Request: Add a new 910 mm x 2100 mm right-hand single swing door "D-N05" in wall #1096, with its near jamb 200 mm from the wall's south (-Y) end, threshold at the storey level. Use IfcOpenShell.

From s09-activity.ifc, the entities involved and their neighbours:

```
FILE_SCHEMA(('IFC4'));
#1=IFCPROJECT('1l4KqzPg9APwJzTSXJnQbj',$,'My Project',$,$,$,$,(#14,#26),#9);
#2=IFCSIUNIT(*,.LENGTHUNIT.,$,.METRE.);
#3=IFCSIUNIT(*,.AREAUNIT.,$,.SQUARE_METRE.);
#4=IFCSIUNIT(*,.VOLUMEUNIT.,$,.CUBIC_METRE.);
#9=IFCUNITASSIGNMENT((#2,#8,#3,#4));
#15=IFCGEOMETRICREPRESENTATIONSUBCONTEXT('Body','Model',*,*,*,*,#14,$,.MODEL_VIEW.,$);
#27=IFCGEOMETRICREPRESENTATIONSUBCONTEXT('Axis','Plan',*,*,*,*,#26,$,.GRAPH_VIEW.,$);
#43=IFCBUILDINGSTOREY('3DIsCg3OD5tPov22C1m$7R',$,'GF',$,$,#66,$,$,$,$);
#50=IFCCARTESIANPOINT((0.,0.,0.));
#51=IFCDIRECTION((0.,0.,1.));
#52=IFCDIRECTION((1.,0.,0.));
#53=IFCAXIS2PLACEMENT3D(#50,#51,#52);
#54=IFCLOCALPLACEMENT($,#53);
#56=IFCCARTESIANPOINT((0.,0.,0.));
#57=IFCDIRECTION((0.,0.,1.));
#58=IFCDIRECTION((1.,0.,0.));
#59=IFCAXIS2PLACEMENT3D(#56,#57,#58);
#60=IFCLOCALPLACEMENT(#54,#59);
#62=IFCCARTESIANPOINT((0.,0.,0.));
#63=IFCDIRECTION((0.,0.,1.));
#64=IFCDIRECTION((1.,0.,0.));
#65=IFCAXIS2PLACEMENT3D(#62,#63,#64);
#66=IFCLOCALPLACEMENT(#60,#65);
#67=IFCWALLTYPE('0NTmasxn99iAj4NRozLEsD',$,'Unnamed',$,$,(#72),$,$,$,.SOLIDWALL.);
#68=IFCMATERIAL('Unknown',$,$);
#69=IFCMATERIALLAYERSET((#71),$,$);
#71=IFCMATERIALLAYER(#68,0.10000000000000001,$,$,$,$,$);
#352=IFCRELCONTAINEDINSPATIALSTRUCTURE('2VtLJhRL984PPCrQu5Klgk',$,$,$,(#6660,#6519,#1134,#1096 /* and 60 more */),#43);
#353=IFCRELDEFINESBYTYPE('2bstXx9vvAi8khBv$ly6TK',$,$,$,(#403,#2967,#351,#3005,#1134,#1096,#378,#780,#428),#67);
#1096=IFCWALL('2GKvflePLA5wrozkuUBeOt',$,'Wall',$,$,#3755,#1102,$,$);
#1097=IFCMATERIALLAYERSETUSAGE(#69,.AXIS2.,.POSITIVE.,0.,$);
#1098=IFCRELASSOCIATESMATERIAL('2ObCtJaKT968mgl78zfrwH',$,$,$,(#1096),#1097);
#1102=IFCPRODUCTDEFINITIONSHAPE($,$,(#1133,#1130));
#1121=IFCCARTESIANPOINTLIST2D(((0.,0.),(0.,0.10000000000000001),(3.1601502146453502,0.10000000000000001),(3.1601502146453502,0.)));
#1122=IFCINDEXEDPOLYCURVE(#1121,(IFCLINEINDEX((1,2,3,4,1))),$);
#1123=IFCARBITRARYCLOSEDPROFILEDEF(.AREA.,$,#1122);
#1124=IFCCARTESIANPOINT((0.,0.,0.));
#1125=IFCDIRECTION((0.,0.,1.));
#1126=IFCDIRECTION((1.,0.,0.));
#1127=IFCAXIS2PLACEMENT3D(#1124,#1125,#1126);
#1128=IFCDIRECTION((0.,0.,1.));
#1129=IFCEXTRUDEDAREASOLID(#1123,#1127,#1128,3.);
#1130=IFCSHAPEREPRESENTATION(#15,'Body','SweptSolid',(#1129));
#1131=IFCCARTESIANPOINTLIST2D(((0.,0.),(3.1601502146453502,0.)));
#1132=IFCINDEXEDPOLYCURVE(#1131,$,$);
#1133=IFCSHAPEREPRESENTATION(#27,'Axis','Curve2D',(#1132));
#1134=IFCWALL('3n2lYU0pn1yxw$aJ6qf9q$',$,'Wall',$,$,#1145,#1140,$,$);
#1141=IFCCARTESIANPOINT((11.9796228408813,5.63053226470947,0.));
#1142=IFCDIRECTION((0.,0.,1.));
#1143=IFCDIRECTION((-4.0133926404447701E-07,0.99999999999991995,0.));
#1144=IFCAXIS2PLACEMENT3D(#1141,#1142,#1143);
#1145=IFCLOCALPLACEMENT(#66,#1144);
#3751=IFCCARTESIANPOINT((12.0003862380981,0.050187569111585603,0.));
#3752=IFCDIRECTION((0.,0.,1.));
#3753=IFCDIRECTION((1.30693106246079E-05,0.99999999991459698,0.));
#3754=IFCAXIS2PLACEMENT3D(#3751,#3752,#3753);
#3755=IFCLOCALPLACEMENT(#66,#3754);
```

```python
import numpy as np
import ifcopenshell
import ifcopenshell.api.feature
import ifcopenshell.api.geometry
import ifcopenshell.api.root
import ifcopenshell.api.spatial
import ifcopenshell.geom
import ifcopenshell.util.element
import ifcopenshell.util.placement
import ifcopenshell.util.representation
import ifcopenshell.util.shape
import ifcopenshell.util.unit

model = ifcopenshell.open("s09-activity.ifc")
unit_scale = ifcopenshell.util.unit.calculate_unit_scale(model)
settings = ifcopenshell.geom.settings()


def volume(element):
    """Net volume in cubic metres, openings subtracted."""
    shape = ifcopenshell.geom.create_shape(settings, element)
    return ifcopenshell.util.shape.get_volume(shape.geometry)


wall = model.by_guid("2GKvflePLA5wrozkuUBeOt")
storey = ifcopenshell.util.element.get_container(wall, ifc_class="IfcBuildingStorey")
context = ifcopenshell.util.representation.get_context(model, "Model", "Body", "MODEL_VIEW")
before = volume(wall)

width, height, from_end, sill = 0.91, 2.1, 0.2, 0.0  # metres

# The wall runs along its own X axis, and the end named is its -X end.
wall_shape = ifcopenshell.geom.create_shape(settings, wall)
x, y, z = ifcopenshell.util.shape.get_vertices(wall_shape.geometry).T
start = x.min() + from_end
face, thickness = float(y.min()), float(y.max() - y.min())
wall_matrix = ifcopenshell.util.placement.get_local_placement(wall.ObjectPlacement)
level = ifcopenshell.util.placement.get_local_placement(storey.ObjectPlacement)[2, 3]


def in_wall(x, y):
    """Placement at x, y metres in the wall's axes, at sill height."""
    matrix = wall_matrix.copy()
    matrix[:, 3] = wall_matrix @ np.array([x / unit_scale, y / unit_scale, 0.0, 1.0])
    matrix[2, 3] = level + sill / unit_scale
    return matrix


# Opening: a box that overshoots both wall faces by 50 mm.
opening = ifcopenshell.api.root.create_entity(model, ifc_class="IfcOpeningElement", predefined_type="OPENING")
box = ifcopenshell.api.geometry.add_wall_representation(
    model, context=context, length=width, height=height, thickness=thickness + 0.1
)
ifcopenshell.api.geometry.assign_representation(model, product=opening, representation=box)
ifcopenshell.api.geometry.edit_object_placement(model, product=opening, matrix=in_wall(start, face - 0.05), is_si=False)
ifcopenshell.api.feature.add_feature(model, feature=opening, element=wall)

door = ifcopenshell.api.root.create_entity(model, ifc_class="IfcDoor", name="D-N05", predefined_type="DOOR")
door.OverallWidth, door.OverallHeight = width / unit_scale, height / unit_scale
door.OperationType = "SINGLE_SWING_RIGHT"
body = ifcopenshell.api.geometry.add_door_representation(
    model,
    context=context,
    overall_width=door.OverallWidth,
    overall_height=door.OverallHeight,
    operation_type="SINGLE_SWING_RIGHT",
    lining_properties={"LiningDepth": thickness / unit_scale, "ThresholdDepth": thickness / unit_scale},
)
ifcopenshell.api.geometry.assign_representation(model, product=door, representation=body)
ifcopenshell.api.spatial.assign_container(model, products=[door], relating_structure=storey)
ifcopenshell.api.feature.add_filling(model, opening=opening, element=door)

# The lining spans the wall, so the door starts at the wall face.
ifcopenshell.api.geometry.edit_object_placement(model, product=door, matrix=in_wall(start, face), is_si=False)

after = volume(wall)

print(f"wall volume {before:.3f} -> {after:.3f} m3")

model.write("s09-activity_rev.ifc")
```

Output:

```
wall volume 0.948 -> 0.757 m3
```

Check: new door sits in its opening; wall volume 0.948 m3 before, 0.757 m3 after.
